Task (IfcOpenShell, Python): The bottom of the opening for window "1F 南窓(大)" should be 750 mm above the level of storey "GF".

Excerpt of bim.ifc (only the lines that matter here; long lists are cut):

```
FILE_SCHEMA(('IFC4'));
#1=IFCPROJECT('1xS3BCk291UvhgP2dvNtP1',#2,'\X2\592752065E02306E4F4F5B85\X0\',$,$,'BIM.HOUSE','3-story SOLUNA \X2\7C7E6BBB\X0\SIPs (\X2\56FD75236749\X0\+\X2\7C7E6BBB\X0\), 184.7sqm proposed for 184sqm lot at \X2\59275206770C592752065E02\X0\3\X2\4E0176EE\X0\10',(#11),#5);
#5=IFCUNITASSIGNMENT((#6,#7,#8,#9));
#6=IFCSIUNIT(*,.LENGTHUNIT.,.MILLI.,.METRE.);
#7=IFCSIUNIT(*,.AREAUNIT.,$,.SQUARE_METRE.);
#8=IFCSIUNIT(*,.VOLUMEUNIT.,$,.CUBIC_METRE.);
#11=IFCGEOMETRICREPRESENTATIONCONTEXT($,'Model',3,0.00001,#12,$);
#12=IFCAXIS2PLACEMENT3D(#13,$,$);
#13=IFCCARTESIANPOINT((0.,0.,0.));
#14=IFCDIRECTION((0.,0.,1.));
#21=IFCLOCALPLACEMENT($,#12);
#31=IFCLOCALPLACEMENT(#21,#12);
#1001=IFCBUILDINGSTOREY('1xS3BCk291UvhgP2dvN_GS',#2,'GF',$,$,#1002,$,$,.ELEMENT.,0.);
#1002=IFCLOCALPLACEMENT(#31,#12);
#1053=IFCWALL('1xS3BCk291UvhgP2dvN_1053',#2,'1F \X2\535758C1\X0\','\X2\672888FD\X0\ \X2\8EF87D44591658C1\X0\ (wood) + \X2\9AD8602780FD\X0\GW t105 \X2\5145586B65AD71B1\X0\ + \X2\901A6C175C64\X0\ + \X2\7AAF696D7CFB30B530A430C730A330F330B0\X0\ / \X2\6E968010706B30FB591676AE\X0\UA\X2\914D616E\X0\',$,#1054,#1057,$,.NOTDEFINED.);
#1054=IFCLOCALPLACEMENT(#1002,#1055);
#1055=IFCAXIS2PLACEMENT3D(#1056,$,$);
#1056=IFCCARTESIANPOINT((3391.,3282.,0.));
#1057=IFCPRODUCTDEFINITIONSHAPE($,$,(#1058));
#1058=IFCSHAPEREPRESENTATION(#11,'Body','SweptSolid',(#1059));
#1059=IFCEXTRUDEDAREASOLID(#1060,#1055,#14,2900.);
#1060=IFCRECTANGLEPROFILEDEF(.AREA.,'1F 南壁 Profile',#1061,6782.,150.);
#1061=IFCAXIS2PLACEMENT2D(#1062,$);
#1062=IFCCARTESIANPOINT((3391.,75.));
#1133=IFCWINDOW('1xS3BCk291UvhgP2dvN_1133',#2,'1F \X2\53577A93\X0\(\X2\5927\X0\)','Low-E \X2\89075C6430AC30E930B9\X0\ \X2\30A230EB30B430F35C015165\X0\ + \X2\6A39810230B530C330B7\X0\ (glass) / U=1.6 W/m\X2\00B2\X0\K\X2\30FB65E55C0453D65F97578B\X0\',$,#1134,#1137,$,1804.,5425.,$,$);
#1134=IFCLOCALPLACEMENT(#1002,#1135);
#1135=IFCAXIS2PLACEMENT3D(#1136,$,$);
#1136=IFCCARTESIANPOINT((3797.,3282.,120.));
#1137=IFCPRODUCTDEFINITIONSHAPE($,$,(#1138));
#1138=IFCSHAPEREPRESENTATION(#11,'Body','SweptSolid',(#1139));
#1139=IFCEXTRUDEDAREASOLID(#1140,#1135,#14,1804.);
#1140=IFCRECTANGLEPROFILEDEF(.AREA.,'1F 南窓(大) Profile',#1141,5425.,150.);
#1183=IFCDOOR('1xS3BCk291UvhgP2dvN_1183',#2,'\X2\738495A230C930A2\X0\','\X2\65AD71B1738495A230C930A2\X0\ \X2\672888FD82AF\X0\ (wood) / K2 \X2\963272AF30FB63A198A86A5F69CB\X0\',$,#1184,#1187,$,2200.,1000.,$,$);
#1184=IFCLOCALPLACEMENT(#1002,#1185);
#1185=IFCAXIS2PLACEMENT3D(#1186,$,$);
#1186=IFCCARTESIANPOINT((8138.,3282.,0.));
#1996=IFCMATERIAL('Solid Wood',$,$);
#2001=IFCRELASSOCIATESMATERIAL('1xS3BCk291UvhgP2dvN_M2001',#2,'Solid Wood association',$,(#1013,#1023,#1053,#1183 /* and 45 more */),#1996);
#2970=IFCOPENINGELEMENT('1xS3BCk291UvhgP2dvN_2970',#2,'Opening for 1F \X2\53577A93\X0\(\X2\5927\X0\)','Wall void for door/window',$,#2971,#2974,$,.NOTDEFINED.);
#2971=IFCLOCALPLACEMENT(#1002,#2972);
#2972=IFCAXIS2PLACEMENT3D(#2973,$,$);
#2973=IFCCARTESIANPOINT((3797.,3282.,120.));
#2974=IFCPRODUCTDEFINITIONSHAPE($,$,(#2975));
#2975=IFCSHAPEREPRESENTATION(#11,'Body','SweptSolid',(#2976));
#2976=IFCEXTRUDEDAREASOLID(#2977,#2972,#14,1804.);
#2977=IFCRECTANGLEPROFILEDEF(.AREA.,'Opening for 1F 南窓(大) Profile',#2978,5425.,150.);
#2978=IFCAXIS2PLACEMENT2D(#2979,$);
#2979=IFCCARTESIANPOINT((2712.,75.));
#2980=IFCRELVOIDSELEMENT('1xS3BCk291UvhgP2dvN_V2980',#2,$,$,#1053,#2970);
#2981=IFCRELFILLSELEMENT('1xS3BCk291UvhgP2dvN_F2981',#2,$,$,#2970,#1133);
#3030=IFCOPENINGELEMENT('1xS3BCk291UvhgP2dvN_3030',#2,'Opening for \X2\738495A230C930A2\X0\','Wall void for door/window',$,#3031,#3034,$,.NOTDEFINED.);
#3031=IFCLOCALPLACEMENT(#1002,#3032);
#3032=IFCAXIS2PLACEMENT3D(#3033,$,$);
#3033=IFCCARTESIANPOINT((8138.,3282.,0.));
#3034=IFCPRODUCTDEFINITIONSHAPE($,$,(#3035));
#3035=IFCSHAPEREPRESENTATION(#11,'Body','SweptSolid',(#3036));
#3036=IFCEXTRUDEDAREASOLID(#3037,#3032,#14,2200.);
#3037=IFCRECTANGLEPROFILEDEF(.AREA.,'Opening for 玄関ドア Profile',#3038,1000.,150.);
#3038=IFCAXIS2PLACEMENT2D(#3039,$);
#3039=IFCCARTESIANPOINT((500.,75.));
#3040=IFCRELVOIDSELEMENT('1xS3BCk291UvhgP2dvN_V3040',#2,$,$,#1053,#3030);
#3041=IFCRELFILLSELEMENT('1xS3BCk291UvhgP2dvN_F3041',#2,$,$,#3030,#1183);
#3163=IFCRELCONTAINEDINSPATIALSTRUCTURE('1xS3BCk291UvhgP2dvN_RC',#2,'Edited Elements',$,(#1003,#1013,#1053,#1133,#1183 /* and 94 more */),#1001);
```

```python
import numpy as np
import ifcopenshell
import ifcopenshell.api.geometry
import ifcopenshell.geom
import ifcopenshell.util.element
import ifcopenshell.util.placement
import ifcopenshell.util.shape
import ifcopenshell.util.unit

model = ifcopenshell.open("bim.ifc")
unit_scale = ifcopenshell.util.unit.calculate_unit_scale(model)

window = model.by_id(1133)
opening = window.FillsVoids[0].RelatingOpeningElement
storey = ifcopenshell.util.element.get_container(window, ifc_class="IfcBuildingStorey")
level = ifcopenshell.util.placement.get_local_placement(storey.ObjectPlacement)[2, 3]

# The opening's origin need not be at the sill, so measure its lowest point.
shape = ifcopenshell.geom.create_shape(ifcopenshell.geom.settings(), opening)
bottom = ifcopenshell.util.shape.get_shape_bottom_elevation(shape, shape.geometry) / unit_scale
dz = level + 750.0 - bottom

shift = np.array([0.0, 0.0, dz])
# The window is not placed relative to its opening, so move both.
for product in (opening, window):
    matrix = ifcopenshell.util.placement.get_local_placement(product.ObjectPlacement)
    matrix[:3, 3] += shift
    ifcopenshell.api.geometry.edit_object_placement(model, product=product, matrix=matrix, is_si=False)

print(f"moved by {dz * unit_scale:+.3f} m")

model.write("bim_edited.ifc")
```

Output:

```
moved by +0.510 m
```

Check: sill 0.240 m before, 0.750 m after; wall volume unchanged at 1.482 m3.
